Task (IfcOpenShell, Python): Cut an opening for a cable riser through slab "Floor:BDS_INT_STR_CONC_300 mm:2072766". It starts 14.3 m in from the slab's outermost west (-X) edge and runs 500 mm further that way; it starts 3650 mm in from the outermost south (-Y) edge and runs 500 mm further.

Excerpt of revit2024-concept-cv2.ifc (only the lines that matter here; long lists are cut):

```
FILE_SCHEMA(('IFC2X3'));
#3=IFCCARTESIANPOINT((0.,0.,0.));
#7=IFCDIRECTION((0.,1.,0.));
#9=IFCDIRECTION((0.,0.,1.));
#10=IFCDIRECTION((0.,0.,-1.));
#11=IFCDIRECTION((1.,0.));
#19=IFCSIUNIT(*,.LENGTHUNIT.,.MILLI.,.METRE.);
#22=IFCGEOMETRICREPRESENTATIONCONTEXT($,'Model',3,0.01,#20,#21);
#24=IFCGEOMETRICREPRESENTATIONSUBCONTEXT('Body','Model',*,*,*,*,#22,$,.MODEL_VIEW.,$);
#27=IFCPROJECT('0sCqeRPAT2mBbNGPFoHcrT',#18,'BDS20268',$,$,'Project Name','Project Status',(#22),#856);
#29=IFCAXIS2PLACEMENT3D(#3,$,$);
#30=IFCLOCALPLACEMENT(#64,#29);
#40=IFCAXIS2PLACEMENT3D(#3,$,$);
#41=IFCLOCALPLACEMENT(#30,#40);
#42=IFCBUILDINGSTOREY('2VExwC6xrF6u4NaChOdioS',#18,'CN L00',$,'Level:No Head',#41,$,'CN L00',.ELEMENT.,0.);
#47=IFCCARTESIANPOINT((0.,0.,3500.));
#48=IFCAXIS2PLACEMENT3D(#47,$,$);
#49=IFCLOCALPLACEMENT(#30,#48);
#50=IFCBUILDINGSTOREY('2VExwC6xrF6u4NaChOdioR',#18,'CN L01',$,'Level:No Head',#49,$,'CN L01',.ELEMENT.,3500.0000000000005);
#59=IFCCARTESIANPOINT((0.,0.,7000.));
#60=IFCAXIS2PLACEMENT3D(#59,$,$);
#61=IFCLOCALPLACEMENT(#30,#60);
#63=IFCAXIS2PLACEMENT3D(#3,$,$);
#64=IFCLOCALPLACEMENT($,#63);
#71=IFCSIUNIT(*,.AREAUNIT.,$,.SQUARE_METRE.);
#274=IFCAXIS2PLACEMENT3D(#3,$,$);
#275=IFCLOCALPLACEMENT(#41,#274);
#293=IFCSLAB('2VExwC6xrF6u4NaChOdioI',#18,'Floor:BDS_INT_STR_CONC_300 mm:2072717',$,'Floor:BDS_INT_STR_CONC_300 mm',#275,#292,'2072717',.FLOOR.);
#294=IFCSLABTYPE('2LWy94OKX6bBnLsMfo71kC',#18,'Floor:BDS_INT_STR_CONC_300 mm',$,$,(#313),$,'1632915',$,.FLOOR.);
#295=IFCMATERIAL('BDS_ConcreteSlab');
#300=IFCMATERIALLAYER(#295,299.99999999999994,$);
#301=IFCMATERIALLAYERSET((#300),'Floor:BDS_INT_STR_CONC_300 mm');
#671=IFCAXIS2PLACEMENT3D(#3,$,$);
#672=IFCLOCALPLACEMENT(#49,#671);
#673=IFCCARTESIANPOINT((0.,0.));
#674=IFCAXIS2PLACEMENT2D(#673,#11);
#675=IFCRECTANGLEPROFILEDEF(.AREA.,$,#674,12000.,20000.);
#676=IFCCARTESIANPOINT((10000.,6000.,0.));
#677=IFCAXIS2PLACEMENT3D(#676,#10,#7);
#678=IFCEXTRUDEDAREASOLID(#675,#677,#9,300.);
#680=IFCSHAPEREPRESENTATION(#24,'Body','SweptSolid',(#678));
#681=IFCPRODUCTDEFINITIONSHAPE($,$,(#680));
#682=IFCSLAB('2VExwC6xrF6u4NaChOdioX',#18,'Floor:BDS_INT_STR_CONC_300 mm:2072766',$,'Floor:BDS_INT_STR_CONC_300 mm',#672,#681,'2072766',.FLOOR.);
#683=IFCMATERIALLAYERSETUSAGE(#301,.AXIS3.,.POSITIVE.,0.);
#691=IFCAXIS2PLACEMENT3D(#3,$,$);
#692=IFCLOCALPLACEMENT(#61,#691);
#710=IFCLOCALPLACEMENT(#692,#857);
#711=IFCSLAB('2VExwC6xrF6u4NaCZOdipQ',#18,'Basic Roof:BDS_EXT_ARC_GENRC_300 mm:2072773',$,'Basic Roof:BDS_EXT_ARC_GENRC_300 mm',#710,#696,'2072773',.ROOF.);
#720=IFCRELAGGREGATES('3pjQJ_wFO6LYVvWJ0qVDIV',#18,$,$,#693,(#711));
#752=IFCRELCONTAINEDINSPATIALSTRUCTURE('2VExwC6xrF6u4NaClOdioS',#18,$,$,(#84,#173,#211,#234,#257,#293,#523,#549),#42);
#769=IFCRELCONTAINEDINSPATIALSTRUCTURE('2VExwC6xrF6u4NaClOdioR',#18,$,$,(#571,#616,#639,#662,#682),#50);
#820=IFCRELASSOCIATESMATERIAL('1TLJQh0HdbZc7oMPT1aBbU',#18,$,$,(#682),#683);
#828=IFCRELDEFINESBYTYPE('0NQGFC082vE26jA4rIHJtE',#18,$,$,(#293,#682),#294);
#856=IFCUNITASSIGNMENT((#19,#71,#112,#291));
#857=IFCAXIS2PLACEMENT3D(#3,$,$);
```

```python
import numpy as np
import ifcopenshell
import ifcopenshell.api.feature
import ifcopenshell.api.geometry
import ifcopenshell.api.root
import ifcopenshell.geom
import ifcopenshell.util.placement
import ifcopenshell.util.representation
import ifcopenshell.util.shape
import ifcopenshell.util.unit

model = ifcopenshell.open("revit2024-concept-cv2.ifc")
unit_scale = ifcopenshell.util.unit.calculate_unit_scale(model)
settings = ifcopenshell.geom.settings()


def volume(element):
    """Net volume in cubic metres, openings subtracted."""
    shape = ifcopenshell.geom.create_shape(settings, element)
    return ifcopenshell.util.shape.get_volume(shape.geometry)


slab = model.by_id(682)
before = volume(slab)

# Extent in the slab's own axes, in metres. The edges named are its -X and -Y sides.
slab_shape = ifcopenshell.geom.create_shape(settings, slab)
vertices = ifcopenshell.util.shape.get_vertices(slab_shape.geometry)
x_min, y_min, bottom = vertices.min(axis=0)
top = vertices[:, 2].max()

opening = ifcopenshell.api.root.create_entity(model, ifc_class="IfcOpeningElement", name="Cable riser opening")
context = ifcopenshell.util.representation.get_context(model, "Model", "Body", "MODEL_VIEW")
width, depth = 0.5, 0.5
outline = [(0.0, 0.0), (width, 0.0), (width, depth), (0.0, depth), (0.0, 0.0)]
# Overshoot both faces by 50 mm so the cut is clean.
shape = ifcopenshell.api.geometry.add_slab_representation(
    model, context=context, depth=top - bottom + 0.1, polyline=outline
)
ifcopenshell.api.geometry.assign_representation(model, product=opening, representation=shape)

matrix = ifcopenshell.util.placement.get_local_placement(slab.ObjectPlacement)
matrix[:, 3] = matrix @ np.append(np.array([x_min + 14.3, y_min + 3.65, bottom - 0.05]) / unit_scale, 1.0)
ifcopenshell.api.geometry.edit_object_placement(model, product=opening, matrix=matrix, is_si=False)
ifcopenshell.api.feature.add_feature(model, feature=opening, element=slab)

after = volume(slab)

print(f"slab volume {before:.3f} -> {after:.3f} m3")

model.write("revit2024-concept-cv2_updated.ifc")
```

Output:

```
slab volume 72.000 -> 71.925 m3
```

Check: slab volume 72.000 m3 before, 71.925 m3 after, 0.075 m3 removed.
